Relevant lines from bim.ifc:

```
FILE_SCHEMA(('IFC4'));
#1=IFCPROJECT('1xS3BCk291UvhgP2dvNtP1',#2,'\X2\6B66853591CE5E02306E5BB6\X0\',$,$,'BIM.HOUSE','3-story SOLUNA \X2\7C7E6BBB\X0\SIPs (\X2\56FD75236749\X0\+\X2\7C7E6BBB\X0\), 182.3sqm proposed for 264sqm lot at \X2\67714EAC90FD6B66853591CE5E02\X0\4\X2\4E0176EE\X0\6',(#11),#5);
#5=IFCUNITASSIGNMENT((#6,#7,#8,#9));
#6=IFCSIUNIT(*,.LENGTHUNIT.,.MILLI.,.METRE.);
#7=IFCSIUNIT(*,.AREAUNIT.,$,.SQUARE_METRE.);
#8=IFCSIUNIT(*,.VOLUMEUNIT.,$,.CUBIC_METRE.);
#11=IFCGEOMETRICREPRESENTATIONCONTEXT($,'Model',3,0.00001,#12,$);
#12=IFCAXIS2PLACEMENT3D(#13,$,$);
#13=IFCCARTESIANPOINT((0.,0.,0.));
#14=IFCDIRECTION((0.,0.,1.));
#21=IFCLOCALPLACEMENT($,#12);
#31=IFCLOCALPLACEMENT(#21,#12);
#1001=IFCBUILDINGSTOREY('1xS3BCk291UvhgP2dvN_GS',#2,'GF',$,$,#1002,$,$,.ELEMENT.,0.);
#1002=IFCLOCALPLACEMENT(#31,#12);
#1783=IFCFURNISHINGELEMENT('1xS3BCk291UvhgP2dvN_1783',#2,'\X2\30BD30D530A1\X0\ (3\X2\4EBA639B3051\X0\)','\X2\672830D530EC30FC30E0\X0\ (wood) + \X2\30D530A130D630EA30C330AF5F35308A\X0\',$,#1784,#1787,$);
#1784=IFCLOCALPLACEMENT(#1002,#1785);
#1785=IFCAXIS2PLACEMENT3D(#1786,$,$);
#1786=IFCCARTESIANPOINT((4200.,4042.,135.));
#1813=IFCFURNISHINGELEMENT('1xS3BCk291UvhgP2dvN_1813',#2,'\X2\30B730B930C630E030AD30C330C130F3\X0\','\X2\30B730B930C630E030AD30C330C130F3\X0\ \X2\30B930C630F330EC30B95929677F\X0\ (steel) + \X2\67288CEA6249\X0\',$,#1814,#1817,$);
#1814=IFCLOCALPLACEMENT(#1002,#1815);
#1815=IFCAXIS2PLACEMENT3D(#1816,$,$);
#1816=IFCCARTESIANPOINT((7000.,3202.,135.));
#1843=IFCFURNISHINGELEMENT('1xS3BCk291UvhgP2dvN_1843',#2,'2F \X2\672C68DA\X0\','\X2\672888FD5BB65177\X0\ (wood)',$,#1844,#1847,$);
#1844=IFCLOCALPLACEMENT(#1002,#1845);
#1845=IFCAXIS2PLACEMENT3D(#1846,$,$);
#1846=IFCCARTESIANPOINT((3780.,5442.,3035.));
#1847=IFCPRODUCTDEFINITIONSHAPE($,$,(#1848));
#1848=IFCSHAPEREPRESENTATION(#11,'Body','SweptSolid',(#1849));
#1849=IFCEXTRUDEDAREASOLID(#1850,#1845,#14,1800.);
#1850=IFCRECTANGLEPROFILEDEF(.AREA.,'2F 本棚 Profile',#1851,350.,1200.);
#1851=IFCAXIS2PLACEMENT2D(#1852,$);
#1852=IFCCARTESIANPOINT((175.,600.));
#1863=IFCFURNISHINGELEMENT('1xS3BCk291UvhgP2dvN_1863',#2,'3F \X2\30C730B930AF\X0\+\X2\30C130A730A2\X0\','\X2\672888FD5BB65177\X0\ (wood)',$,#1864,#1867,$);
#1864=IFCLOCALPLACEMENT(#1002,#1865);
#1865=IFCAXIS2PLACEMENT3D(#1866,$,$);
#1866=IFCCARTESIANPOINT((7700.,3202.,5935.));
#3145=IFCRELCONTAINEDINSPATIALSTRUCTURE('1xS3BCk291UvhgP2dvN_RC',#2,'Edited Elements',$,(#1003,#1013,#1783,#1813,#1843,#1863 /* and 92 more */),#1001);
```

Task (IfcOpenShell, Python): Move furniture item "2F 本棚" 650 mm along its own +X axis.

```python
import ifcopenshell
import ifcopenshell.api.geometry
import ifcopenshell.util.placement

model = ifcopenshell.open("bim.ifc")

item = model.by_id(1843)
matrix = ifcopenshell.util.placement.get_local_placement(item.ObjectPlacement)
matrix[:3, 3] += matrix[:3, 0] * 650.0
ifcopenshell.api.geometry.edit_object_placement(model, product=item, matrix=matrix, is_si=False)

print(ifcopenshell.util.placement.get_local_placement(item.ObjectPlacement).round(3) + 0.0)

model.write("bim_rev.ifc")
```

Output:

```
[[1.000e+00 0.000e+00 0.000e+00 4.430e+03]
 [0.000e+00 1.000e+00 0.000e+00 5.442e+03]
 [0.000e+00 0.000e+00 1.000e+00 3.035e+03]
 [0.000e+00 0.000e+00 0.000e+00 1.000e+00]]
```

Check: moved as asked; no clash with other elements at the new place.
